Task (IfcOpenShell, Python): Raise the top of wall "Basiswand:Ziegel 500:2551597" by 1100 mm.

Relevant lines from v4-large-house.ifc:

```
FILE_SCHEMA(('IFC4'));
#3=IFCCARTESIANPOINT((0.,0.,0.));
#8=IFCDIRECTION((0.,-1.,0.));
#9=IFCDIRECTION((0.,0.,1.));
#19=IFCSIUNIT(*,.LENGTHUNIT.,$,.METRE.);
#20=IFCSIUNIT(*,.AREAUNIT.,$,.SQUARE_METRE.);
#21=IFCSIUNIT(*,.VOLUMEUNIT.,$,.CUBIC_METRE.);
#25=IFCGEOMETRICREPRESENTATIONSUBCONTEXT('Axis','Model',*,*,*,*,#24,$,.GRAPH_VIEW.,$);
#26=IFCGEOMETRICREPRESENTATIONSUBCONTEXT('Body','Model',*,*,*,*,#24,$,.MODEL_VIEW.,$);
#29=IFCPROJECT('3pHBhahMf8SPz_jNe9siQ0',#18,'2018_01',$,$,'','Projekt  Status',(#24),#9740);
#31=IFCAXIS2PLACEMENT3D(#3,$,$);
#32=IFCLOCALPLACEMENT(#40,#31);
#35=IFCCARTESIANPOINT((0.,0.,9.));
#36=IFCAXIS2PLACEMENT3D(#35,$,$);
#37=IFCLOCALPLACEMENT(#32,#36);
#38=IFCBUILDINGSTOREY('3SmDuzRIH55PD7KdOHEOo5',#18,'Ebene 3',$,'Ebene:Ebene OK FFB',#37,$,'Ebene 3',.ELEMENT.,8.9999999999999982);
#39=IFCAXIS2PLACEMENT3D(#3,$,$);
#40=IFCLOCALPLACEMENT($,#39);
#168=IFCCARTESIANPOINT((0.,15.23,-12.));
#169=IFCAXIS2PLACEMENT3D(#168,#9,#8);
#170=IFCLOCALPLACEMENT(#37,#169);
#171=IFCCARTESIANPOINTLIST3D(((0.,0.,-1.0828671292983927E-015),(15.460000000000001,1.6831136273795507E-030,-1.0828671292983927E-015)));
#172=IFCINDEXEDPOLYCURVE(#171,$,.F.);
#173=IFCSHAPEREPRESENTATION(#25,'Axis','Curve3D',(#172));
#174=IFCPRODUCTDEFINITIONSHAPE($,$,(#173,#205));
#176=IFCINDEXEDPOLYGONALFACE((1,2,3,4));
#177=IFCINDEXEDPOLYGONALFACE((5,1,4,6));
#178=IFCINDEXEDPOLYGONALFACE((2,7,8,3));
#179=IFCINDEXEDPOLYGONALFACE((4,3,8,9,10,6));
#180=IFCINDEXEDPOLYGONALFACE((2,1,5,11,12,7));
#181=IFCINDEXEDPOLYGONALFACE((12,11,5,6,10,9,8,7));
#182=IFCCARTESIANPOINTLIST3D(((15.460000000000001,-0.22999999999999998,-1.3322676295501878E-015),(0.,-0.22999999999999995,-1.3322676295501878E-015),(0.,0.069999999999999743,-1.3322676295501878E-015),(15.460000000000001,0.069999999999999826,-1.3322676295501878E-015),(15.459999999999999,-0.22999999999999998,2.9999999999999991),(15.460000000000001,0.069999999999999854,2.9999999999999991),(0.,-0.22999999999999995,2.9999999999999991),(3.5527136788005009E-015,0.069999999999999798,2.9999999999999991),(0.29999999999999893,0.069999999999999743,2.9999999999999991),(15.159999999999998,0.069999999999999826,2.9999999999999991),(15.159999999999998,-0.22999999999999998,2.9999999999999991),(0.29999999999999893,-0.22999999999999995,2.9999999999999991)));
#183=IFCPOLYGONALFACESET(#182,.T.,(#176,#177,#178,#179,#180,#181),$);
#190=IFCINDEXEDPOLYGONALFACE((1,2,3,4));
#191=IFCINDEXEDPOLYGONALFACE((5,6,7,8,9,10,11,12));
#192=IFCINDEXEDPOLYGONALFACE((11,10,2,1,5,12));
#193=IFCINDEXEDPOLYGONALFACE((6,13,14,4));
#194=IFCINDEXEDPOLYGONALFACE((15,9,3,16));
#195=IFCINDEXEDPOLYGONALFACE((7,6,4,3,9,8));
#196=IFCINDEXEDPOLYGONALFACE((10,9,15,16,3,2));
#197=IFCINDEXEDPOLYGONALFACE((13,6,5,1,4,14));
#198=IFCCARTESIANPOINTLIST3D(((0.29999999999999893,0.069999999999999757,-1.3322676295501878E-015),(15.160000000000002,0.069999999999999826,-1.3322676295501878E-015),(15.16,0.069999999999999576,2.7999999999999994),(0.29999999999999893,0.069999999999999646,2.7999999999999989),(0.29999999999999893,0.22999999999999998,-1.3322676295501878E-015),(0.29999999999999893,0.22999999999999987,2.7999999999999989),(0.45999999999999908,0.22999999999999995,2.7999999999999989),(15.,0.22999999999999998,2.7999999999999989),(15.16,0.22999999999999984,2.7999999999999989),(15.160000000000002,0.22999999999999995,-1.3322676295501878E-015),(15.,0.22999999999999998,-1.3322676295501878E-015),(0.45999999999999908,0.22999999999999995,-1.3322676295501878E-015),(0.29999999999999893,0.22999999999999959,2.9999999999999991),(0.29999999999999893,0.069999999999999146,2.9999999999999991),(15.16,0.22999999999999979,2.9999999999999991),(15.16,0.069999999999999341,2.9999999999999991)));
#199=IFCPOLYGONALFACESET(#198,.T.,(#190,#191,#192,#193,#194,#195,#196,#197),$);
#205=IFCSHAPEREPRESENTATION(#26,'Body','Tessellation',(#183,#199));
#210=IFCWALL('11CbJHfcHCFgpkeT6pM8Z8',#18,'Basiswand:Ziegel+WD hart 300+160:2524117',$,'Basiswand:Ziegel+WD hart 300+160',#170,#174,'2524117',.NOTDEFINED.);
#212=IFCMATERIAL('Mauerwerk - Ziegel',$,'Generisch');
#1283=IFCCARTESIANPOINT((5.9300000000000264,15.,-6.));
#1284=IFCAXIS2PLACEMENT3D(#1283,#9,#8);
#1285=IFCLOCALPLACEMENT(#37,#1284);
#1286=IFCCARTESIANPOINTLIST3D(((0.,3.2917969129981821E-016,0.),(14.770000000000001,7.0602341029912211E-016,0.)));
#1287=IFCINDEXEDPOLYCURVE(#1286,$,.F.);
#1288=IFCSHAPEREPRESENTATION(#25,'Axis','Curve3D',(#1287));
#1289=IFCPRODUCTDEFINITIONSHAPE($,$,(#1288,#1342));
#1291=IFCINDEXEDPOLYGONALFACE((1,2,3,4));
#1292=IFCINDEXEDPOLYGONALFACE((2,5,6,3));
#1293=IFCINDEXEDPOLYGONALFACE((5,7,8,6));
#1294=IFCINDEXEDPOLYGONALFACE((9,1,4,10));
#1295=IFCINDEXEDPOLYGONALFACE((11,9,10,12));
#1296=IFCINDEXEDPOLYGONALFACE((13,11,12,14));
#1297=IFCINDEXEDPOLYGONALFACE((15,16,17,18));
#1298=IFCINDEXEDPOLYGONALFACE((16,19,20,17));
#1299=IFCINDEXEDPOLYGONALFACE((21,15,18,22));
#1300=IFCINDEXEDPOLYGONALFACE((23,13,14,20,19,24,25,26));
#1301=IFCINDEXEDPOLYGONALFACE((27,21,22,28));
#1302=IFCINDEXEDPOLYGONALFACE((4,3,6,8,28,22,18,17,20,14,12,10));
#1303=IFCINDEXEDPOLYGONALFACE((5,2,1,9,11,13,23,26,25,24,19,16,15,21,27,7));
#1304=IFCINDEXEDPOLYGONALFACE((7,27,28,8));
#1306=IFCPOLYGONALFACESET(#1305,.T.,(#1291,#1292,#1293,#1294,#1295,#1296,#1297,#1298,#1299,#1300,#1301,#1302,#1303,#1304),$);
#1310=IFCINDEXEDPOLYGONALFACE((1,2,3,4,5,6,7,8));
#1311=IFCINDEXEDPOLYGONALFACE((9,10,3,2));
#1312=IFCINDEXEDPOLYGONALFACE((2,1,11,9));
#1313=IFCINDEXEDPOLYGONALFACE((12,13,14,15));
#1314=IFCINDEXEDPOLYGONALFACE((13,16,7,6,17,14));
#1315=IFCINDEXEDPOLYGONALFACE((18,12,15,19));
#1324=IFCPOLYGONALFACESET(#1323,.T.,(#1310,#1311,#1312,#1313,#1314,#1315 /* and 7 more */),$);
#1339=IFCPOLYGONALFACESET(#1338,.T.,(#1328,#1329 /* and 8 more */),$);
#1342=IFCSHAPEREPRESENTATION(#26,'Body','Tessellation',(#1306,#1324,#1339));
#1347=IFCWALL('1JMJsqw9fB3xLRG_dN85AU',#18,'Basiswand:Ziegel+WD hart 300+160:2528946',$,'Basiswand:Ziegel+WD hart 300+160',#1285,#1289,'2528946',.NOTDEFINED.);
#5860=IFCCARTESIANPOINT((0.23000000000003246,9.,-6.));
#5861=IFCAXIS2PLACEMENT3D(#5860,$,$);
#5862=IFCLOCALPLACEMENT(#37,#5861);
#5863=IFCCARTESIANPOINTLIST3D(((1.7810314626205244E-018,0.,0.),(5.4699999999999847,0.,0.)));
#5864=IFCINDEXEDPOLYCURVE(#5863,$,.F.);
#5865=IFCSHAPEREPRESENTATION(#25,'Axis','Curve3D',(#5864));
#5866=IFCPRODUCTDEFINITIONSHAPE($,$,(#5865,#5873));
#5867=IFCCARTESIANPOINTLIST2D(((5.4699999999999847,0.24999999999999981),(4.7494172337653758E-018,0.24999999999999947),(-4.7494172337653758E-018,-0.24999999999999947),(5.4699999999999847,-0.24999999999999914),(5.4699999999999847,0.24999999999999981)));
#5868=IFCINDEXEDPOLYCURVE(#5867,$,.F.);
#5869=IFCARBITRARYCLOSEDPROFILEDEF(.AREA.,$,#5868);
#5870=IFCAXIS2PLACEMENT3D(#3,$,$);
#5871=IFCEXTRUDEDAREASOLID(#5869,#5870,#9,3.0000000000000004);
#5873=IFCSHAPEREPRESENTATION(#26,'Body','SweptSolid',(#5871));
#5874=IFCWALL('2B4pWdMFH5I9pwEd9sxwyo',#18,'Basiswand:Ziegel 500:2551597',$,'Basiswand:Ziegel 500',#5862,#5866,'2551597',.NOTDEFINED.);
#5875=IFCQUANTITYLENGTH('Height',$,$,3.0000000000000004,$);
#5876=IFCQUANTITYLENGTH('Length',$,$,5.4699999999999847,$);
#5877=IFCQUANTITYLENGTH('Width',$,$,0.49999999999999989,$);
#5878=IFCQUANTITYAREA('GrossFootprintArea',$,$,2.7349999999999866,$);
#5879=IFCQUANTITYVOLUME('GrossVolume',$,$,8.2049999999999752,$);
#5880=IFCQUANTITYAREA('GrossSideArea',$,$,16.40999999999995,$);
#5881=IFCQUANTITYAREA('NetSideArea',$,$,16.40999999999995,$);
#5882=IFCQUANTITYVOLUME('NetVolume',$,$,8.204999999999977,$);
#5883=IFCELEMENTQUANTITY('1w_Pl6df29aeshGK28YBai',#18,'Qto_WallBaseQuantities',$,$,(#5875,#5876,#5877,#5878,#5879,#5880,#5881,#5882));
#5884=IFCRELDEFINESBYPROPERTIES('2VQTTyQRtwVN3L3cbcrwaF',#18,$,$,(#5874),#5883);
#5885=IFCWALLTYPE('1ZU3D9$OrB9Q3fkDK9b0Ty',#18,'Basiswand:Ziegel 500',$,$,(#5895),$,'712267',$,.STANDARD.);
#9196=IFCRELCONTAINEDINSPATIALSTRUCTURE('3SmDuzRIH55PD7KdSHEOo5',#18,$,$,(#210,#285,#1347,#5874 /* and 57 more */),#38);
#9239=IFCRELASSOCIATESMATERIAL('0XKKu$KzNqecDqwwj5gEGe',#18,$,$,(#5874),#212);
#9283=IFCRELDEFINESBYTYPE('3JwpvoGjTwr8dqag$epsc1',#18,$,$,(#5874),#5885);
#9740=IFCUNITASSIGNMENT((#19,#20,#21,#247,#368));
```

```python
import ifcopenshell
import ifcopenshell.api.pset
import ifcopenshell.geom
import ifcopenshell.util.element
import ifcopenshell.util.representation
import ifcopenshell.util.shape
import ifcopenshell.util.unit

model = ifcopenshell.open("v4-large-house.ifc")
unit_scale = ifcopenshell.util.unit.calculate_unit_scale(model)
area_scale = ifcopenshell.util.unit.calculate_unit_scale(model, "AREAUNIT")
volume_scale = ifcopenshell.util.unit.calculate_unit_scale(model, "VOLUMEUNIT")
settings = ifcopenshell.geom.settings()


def volume(element):
    """Net volume in cubic metres, openings subtracted."""
    shape = ifcopenshell.geom.create_shape(settings, element)
    return ifcopenshell.util.shape.get_volume(shape.geometry)


wall = model.by_id(5874)
before = volume(wall)

body = ifcopenshell.util.representation.get_representation(wall, "Model", "Body")
solid = body.Items[0]
old_height = solid.Depth
solid.Depth += 1.1 / unit_scale
after = volume(wall)
thickness = 0.5  # wall thickness in metres

# Update the stored height, areas and volumes.
qto = model.by_id(ifcopenshell.util.element.get_pset(wall, "Qto_WallBaseQuantities", should_inherit=False)["id"])
ifcopenshell.api.pset.edit_qto(model, qto=qto, properties={
    "Height": solid.Depth,
    "GrossVolume": ifcopenshell.util.element.get_pset(wall, "Qto_WallBaseQuantities", "GrossVolume") * solid.Depth / old_height,
    "GrossSideArea": ifcopenshell.util.element.get_pset(wall, "Qto_WallBaseQuantities", "GrossSideArea") * solid.Depth / old_height,
    "NetSideArea": after / thickness / area_scale,
    "NetVolume": after / volume_scale,
})

print(f"height {old_height:g} -> {solid.Depth:g}, volume {before:.3f} -> {after:.3f} m3")

model.write("v4-large-house_edited.ifc")
```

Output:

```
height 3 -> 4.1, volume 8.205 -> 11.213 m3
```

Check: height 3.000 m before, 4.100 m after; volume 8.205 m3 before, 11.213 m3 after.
